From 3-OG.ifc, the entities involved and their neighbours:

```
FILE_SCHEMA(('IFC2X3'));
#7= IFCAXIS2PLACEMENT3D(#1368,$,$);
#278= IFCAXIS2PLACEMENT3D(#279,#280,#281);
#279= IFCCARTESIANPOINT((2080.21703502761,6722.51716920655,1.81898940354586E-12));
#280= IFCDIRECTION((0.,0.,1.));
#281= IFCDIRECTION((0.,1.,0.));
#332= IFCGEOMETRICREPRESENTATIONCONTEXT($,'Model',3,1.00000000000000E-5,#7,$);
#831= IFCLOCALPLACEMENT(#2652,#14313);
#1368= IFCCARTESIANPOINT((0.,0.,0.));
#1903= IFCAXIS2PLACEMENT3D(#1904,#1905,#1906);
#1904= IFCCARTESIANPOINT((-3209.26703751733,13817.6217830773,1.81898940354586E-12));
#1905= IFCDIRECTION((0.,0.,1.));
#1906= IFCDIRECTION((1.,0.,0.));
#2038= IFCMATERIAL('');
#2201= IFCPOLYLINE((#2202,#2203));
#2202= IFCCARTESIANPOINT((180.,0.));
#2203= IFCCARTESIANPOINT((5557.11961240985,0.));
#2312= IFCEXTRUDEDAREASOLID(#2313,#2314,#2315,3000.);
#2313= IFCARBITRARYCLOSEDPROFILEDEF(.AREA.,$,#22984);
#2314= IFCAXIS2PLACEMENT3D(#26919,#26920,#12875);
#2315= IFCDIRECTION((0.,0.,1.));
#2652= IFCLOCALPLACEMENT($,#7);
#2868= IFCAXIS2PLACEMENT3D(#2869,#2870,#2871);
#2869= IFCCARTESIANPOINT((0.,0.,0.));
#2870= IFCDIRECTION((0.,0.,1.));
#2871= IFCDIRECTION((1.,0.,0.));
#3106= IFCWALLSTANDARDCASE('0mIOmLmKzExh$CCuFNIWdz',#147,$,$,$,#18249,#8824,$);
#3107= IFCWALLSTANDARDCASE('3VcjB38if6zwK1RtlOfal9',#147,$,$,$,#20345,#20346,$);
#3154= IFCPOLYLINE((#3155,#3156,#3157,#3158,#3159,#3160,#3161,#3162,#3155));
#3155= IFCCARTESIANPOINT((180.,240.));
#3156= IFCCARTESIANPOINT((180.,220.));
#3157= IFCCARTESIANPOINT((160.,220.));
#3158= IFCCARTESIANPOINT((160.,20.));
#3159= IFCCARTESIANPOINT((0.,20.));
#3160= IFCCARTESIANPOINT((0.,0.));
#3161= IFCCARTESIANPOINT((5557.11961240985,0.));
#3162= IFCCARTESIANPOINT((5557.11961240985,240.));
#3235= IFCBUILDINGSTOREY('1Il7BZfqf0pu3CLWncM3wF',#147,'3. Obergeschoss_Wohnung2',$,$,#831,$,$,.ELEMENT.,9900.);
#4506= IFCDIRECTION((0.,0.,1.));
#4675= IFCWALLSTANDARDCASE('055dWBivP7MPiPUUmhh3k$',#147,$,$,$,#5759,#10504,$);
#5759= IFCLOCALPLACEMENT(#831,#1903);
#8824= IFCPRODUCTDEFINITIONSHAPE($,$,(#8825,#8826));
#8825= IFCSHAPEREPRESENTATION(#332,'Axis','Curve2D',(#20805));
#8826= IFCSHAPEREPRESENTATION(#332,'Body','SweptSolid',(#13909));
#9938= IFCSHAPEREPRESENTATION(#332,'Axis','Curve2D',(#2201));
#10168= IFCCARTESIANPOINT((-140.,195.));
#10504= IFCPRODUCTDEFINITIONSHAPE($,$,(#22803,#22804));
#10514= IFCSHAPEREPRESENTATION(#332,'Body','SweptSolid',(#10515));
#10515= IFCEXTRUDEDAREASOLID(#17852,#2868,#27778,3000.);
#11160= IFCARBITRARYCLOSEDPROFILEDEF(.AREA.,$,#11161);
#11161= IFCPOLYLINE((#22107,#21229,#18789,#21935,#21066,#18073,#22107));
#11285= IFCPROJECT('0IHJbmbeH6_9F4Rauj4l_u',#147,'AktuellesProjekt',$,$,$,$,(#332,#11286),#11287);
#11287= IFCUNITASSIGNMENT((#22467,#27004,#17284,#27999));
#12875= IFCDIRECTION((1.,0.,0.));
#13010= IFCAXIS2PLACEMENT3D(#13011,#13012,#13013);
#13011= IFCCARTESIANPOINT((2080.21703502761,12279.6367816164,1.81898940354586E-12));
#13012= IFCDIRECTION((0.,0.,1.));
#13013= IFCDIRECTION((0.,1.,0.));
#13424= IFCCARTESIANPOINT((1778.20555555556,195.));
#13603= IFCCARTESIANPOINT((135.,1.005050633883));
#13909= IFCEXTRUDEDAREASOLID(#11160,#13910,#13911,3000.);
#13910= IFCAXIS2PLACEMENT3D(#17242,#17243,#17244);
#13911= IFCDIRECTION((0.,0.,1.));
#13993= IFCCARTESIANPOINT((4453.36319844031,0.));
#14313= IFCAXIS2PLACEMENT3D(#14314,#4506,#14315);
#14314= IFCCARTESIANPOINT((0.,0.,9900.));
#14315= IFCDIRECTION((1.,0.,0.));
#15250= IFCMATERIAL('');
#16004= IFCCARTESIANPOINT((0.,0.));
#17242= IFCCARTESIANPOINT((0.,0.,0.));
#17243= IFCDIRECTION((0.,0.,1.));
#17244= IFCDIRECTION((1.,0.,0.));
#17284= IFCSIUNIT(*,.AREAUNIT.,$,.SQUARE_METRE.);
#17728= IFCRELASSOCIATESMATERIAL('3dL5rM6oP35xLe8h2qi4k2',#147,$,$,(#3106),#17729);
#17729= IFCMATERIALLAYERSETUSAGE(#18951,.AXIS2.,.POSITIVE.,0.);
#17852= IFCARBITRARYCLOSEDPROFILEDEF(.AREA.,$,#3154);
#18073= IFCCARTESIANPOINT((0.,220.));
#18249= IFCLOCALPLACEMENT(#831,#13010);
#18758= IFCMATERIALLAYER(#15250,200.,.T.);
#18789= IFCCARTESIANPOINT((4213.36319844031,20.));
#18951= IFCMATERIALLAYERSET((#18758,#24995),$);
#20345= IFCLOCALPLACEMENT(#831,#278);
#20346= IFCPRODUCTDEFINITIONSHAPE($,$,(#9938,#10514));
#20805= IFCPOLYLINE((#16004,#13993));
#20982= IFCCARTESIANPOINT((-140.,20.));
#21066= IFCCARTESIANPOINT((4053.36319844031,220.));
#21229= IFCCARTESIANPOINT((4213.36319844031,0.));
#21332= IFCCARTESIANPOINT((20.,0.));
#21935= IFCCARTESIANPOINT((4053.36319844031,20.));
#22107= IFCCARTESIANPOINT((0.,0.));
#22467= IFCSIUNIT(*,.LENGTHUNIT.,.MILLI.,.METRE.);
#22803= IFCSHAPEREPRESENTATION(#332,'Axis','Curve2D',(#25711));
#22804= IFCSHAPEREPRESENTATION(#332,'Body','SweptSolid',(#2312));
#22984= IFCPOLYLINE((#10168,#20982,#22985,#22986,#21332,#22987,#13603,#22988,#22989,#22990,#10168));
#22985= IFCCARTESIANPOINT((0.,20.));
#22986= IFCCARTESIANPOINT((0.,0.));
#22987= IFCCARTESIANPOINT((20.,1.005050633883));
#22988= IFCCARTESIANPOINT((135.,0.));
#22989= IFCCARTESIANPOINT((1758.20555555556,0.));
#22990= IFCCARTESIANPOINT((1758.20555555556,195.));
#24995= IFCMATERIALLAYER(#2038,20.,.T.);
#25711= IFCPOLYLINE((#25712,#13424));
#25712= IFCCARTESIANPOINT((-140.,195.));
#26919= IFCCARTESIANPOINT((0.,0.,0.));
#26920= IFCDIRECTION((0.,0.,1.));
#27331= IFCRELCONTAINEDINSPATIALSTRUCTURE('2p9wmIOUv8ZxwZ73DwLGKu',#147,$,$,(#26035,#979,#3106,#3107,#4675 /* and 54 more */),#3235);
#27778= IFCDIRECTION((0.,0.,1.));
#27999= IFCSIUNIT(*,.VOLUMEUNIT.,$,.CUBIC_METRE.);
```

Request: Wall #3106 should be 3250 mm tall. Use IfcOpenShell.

```python
import ifcopenshell
import ifcopenshell.geom
import ifcopenshell.util.shape

model = ifcopenshell.open("3-OG.ifc")
settings = ifcopenshell.geom.settings()


def volume(element):
    """Net volume in cubic metres, openings subtracted."""
    shape = ifcopenshell.geom.create_shape(settings, element)
    return ifcopenshell.util.shape.get_volume(shape.geometry)


wall = model.by_guid("0mIOmLmKzExh$CCuFNIWdz")
before = volume(wall)

body = next(r for r in wall.Representation.Representations if r.RepresentationIdentifier == "Body")
solid = body.Items[0]
old_height = solid.Depth
solid.Depth = 3250.0
after = volume(wall)

print(f"height {old_height:g} -> {solid.Depth:g}, volume {before:.3f} -> {after:.3f} m3")

model.write("3-OG_v2.ifc")
```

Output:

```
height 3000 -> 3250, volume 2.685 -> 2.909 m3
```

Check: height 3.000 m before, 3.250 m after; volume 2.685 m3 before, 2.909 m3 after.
